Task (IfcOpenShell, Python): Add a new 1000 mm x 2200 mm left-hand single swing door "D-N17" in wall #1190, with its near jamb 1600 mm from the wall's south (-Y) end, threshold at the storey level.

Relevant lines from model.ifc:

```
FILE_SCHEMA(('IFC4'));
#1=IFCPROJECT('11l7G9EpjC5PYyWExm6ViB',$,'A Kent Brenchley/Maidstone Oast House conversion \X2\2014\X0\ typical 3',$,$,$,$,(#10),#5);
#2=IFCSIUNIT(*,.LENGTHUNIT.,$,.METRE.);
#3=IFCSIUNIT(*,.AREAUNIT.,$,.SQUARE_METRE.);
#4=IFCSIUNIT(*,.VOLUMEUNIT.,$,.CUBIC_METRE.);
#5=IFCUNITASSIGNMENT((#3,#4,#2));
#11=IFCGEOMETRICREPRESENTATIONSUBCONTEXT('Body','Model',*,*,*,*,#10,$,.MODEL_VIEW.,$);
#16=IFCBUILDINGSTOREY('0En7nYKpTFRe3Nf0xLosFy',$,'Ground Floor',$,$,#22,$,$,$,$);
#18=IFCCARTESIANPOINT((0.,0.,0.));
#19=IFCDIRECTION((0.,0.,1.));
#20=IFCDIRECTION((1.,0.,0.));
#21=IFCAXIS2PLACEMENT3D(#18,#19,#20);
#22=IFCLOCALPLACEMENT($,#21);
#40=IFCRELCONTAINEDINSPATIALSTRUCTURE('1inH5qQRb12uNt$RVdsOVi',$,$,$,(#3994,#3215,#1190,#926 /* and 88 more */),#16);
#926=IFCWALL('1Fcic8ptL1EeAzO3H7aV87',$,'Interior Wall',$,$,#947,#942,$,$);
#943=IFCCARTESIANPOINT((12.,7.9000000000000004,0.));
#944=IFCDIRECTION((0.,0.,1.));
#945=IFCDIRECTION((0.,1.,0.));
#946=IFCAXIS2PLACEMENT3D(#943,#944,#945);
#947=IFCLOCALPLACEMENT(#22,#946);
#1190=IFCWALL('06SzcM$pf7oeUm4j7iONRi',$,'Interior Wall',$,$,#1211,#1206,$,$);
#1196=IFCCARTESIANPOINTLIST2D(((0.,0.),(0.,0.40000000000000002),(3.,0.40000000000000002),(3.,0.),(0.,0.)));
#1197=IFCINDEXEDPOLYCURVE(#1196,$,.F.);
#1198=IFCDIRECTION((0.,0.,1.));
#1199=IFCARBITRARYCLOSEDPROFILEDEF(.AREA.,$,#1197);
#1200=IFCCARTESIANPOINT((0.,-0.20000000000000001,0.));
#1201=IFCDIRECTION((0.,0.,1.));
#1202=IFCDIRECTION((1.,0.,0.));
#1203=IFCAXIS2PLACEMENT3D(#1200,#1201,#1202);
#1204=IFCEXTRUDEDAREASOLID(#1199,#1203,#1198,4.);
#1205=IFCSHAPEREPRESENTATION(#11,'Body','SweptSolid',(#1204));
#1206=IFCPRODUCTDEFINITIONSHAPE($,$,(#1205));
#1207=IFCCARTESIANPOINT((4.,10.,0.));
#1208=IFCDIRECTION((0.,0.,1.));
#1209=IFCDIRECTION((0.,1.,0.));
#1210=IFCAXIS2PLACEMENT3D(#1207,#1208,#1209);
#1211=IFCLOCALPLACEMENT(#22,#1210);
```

```python
import numpy as np
import ifcopenshell
import ifcopenshell.api.feature
import ifcopenshell.api.geometry
import ifcopenshell.api.root
import ifcopenshell.api.spatial
import ifcopenshell.geom
import ifcopenshell.util.element
import ifcopenshell.util.placement
import ifcopenshell.util.representation
import ifcopenshell.util.shape
import ifcopenshell.util.unit

model = ifcopenshell.open("model.ifc")
unit_scale = ifcopenshell.util.unit.calculate_unit_scale(model)
settings = ifcopenshell.geom.settings()


def volume(element):
    """Net volume in cubic metres, openings subtracted."""
    shape = ifcopenshell.geom.create_shape(settings, element)
    return ifcopenshell.util.shape.get_volume(shape.geometry)


wall = model.by_guid("06SzcM$pf7oeUm4j7iONRi")
storey = ifcopenshell.util.element.get_container(wall, ifc_class="IfcBuildingStorey")
context = ifcopenshell.util.representation.get_context(model, "Model", "Body", "MODEL_VIEW")
before = volume(wall)

width, height, from_end, sill = 1, 2.2, 1.6, 0.0  # metres

# The wall runs along its own X axis, and the end named is its -X end.
wall_shape = ifcopenshell.geom.create_shape(settings, wall)
x, y, z = ifcopenshell.util.shape.get_vertices(wall_shape.geometry).T
start = x.min() + from_end
face, thickness = float(y.min()), float(y.max() - y.min())
wall_matrix = ifcopenshell.util.placement.get_local_placement(wall.ObjectPlacement)
level = ifcopenshell.util.placement.get_local_placement(storey.ObjectPlacement)[2, 3]


def in_wall(x, y):
    """Placement at x, y metres in the wall's axes, at sill height."""
    matrix = wall_matrix.copy()
    matrix[:, 3] = wall_matrix @ np.array([x / unit_scale, y / unit_scale, 0.0, 1.0])
    matrix[2, 3] = level + sill / unit_scale
    return matrix


# Opening: a box that overshoots both wall faces by 50 mm.
opening = ifcopenshell.api.root.create_entity(model, ifc_class="IfcOpeningElement", predefined_type="OPENING")
box = ifcopenshell.api.geometry.add_wall_representation(
    model, context=context, length=width, height=height, thickness=thickness + 0.1
)
ifcopenshell.api.geometry.assign_representation(model, product=opening, representation=box)
ifcopenshell.api.geometry.edit_object_placement(model, product=opening, matrix=in_wall(start, face - 0.05), is_si=False)
ifcopenshell.api.feature.add_feature(model, feature=opening, element=wall)

door = ifcopenshell.api.root.create_entity(model, ifc_class="IfcDoor", name="D-N17", predefined_type="DOOR")
door.OverallWidth, door.OverallHeight = width / unit_scale, height / unit_scale
door.OperationType = "SINGLE_SWING_LEFT"
body = ifcopenshell.api.geometry.add_door_representation(
    model,
    context=context,
    overall_width=door.OverallWidth,
    overall_height=door.OverallHeight,
    operation_type="SINGLE_SWING_LEFT",
    lining_properties={"LiningDepth": thickness / unit_scale, "ThresholdDepth": thickness / unit_scale},
)
ifcopenshell.api.geometry.assign_representation(model, product=door, representation=body)
ifcopenshell.api.spatial.assign_container(model, products=[door], relating_structure=storey)
ifcopenshell.api.feature.add_filling(model, opening=opening, element=door)

# The lining spans the wall, so the door starts at the wall face.
ifcopenshell.api.geometry.edit_object_placement(model, product=door, matrix=in_wall(start, face), is_si=False)

after = volume(wall)

print(f"wall volume {before:.3f} -> {after:.3f} m3")

model.write("model-out.ifc")
```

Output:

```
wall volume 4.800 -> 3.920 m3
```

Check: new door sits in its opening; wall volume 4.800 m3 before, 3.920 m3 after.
